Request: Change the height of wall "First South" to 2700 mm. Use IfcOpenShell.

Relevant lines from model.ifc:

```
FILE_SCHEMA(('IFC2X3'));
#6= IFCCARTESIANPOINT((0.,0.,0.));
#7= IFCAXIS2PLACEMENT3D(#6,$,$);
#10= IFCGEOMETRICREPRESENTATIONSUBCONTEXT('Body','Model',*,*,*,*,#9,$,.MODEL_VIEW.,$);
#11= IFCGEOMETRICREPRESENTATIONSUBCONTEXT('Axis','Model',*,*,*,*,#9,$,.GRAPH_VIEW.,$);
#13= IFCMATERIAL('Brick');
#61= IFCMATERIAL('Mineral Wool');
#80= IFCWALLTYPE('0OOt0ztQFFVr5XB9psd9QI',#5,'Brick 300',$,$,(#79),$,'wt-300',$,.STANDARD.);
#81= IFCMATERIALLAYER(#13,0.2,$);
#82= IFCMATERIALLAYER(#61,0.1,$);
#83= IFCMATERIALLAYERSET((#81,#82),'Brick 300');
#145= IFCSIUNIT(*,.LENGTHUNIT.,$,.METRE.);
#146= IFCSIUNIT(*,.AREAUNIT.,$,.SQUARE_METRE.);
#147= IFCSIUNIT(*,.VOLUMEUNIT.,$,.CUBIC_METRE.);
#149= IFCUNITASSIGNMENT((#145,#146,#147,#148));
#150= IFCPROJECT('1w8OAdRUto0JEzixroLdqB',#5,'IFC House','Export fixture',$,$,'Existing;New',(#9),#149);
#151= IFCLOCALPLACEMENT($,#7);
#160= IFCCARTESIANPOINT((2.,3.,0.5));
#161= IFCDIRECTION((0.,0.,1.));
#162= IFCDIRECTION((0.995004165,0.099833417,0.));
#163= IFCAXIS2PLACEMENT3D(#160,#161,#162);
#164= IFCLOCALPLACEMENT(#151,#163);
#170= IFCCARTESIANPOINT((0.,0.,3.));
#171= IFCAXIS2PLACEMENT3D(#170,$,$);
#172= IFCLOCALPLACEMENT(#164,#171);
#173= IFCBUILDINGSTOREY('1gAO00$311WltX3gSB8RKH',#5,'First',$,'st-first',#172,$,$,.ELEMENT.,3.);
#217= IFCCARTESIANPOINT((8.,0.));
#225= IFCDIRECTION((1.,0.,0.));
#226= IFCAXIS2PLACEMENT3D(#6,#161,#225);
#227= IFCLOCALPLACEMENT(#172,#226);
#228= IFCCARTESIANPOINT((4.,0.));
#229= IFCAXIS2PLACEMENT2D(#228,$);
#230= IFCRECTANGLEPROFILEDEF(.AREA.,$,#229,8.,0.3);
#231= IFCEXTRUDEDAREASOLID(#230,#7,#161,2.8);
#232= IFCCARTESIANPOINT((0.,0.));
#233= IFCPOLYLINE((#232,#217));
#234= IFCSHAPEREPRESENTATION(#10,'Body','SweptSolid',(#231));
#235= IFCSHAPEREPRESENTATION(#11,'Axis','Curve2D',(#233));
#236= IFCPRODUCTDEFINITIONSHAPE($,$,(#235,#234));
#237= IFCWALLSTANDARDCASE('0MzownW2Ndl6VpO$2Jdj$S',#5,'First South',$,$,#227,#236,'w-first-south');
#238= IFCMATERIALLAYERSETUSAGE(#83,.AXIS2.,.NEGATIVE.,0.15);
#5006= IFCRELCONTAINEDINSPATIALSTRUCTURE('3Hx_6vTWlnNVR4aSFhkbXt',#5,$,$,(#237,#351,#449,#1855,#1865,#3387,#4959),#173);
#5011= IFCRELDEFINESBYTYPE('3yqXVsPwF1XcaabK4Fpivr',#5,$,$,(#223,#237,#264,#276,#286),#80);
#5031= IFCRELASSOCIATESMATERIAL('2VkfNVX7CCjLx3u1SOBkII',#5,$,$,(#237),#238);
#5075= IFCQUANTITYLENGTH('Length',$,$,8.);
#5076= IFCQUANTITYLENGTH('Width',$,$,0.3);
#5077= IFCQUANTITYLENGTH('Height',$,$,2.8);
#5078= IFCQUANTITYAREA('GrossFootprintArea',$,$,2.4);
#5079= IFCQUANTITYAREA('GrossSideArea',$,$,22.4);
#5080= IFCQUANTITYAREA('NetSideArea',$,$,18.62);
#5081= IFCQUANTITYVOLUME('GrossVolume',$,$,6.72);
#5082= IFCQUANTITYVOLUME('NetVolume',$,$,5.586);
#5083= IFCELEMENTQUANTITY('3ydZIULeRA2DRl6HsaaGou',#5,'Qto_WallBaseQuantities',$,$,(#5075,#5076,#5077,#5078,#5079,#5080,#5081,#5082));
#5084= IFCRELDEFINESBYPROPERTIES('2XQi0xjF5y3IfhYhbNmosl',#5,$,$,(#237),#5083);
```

```python
import ifcopenshell
import ifcopenshell.api.pset
import ifcopenshell.geom
import ifcopenshell.util.element
import ifcopenshell.util.representation
import ifcopenshell.util.shape
import ifcopenshell.util.unit

model = ifcopenshell.open("model.ifc")
unit_scale = ifcopenshell.util.unit.calculate_unit_scale(model)
area_scale = ifcopenshell.util.unit.calculate_unit_scale(model, "AREAUNIT")
volume_scale = ifcopenshell.util.unit.calculate_unit_scale(model, "VOLUMEUNIT")
settings = ifcopenshell.geom.settings()


def volume(element):
    """Net volume in cubic metres, openings subtracted."""
    shape = ifcopenshell.geom.create_shape(settings, element)
    return ifcopenshell.util.shape.get_volume(shape.geometry)


wall = model.by_id(237)
before = volume(wall)

body = ifcopenshell.util.representation.get_representation(wall, "Model", "Body")
solid = body.Items[0]
old_height = solid.Depth
solid.Depth = 2.7
after = volume(wall)
thickness = 0.3  # wall thickness in metres

# Update the stored height, areas and volumes.
qto = model.by_id(ifcopenshell.util.element.get_pset(wall, "Qto_WallBaseQuantities", should_inherit=False)["id"])
ifcopenshell.api.pset.edit_qto(model, qto=qto, properties={
    "Height": solid.Depth,
    "GrossSideArea": ifcopenshell.util.element.get_pset(wall, "Qto_WallBaseQuantities", "GrossSideArea") * solid.Depth / old_height,
    "NetSideArea": after / thickness / area_scale,
    "GrossVolume": ifcopenshell.util.element.get_pset(wall, "Qto_WallBaseQuantities", "GrossVolume") * solid.Depth / old_height,
    "NetVolume": after / volume_scale,
})

print(f"height {old_height:g} -> {solid.Depth:g}, volume {before:.3f} -> {after:.3f} m3")

model.write("model-out.ifc")
```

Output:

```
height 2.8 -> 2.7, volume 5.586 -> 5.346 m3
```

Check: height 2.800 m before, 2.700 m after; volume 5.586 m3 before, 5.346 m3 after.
